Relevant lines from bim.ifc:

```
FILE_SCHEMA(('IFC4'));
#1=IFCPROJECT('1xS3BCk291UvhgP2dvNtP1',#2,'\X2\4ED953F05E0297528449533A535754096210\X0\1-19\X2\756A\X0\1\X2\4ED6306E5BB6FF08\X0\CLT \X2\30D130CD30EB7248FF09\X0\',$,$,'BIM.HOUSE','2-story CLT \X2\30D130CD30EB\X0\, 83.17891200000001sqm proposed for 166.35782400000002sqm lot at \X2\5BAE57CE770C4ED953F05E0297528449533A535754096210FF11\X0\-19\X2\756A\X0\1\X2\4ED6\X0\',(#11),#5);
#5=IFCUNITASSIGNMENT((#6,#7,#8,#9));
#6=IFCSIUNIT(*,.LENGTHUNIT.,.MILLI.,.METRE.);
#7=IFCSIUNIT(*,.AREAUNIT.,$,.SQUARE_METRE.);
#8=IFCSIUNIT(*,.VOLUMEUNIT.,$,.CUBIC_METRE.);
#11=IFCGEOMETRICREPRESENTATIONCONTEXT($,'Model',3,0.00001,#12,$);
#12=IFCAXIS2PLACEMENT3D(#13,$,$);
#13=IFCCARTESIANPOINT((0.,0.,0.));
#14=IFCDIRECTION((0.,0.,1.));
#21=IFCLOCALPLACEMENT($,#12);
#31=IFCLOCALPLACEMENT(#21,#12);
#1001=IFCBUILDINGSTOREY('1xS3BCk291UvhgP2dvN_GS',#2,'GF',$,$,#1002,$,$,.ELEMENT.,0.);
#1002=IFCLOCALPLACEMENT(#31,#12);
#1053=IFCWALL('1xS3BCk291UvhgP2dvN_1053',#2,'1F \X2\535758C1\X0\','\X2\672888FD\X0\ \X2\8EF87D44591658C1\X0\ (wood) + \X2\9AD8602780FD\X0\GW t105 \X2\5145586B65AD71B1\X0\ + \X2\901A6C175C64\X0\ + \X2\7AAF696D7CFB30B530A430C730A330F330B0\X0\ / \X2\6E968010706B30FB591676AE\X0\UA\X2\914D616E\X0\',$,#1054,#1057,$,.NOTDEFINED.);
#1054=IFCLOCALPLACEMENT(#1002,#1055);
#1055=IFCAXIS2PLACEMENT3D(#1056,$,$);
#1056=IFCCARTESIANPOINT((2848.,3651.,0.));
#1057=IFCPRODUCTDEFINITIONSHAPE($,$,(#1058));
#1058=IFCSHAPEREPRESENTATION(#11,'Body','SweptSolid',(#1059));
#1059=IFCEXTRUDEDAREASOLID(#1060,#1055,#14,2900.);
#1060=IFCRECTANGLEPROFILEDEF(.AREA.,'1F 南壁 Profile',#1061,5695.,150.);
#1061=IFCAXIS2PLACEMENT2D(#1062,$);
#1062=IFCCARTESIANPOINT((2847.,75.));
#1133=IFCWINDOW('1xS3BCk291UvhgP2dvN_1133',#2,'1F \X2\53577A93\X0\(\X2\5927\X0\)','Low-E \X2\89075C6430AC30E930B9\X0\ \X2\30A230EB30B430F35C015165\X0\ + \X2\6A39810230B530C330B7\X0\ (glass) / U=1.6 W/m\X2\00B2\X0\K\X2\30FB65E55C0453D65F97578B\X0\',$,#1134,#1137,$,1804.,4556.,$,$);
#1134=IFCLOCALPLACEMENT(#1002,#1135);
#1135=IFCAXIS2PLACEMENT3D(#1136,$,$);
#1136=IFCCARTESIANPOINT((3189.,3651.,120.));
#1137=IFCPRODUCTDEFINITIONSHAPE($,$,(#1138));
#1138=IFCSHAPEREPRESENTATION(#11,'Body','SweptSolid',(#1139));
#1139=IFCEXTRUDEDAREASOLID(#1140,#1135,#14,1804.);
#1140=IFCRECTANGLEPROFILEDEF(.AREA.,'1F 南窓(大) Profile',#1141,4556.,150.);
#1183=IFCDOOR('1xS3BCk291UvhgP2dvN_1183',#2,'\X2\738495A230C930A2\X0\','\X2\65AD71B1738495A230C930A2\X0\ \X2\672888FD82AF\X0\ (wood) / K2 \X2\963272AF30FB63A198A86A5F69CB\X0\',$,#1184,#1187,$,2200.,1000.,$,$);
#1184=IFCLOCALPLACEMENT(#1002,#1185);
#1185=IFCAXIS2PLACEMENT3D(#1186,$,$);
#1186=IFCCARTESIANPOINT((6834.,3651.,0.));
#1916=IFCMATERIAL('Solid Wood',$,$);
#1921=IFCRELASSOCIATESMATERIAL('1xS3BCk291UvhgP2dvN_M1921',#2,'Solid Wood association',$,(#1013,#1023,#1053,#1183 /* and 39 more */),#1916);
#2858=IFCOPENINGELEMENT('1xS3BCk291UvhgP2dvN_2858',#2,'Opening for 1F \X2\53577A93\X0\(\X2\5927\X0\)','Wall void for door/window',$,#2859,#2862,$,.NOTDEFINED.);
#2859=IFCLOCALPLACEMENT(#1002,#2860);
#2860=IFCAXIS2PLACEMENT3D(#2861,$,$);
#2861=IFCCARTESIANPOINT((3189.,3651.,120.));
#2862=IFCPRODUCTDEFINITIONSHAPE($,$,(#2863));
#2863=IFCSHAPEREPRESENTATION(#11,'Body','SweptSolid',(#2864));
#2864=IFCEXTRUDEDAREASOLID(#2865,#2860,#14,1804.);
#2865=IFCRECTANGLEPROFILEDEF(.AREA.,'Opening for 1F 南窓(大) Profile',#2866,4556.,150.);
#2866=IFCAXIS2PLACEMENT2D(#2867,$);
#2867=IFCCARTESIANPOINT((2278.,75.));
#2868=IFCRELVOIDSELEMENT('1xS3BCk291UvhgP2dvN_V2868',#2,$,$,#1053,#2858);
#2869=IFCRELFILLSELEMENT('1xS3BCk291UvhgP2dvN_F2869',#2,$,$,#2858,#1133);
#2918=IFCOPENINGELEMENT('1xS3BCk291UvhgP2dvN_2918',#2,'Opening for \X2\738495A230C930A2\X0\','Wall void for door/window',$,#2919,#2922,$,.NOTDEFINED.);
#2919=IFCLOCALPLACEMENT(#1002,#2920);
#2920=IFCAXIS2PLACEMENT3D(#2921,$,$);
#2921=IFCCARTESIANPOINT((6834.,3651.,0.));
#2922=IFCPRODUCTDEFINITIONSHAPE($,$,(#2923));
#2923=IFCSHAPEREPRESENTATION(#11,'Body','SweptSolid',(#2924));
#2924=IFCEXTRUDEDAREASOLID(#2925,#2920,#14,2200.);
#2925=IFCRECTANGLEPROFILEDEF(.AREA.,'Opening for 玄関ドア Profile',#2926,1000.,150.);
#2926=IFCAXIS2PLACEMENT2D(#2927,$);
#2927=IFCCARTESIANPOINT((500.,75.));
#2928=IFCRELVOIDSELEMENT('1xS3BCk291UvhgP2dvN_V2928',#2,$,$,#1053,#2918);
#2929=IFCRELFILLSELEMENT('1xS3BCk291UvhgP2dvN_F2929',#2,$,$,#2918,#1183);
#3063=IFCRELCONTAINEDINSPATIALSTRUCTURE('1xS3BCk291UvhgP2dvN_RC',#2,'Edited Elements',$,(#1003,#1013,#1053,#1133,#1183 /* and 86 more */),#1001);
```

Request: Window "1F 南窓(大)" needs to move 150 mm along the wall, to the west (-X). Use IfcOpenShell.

```python
import ifcopenshell
import ifcopenshell.api.geometry
import ifcopenshell.util.placement

model = ifcopenshell.open("bim.ifc")

window = model.by_id(1133)
opening = window.FillsVoids[0].RelatingOpeningElement
wall = opening.VoidsElements[0].RelatingBuildingElement

wall_matrix = ifcopenshell.util.placement.get_local_placement(wall.ObjectPlacement)
shift = wall_matrix[:3, 0] * -150.0
before = ifcopenshell.util.placement.get_local_placement(window.ObjectPlacement)[:3, 3].copy()

# The window is not placed relative to its opening, so move both.
for product in (opening, window):
    matrix = ifcopenshell.util.placement.get_local_placement(product.ObjectPlacement)
    matrix[:3, 3] += shift
    ifcopenshell.api.geometry.edit_object_placement(model, product=product, matrix=matrix, is_si=False)

after = ifcopenshell.util.placement.get_local_placement(window.ObjectPlacement)[:3, 3]
print("window moved by", (after - before).round(3) + 0.0)

model.write("bim-out.ifc")
```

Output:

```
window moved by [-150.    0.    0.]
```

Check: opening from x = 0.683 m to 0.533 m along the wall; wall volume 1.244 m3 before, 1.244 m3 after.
